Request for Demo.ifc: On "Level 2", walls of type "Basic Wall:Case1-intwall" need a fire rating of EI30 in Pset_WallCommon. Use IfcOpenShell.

First a look at what the model holds.

```python
import ifcopenshell
import ifcopenshell.util.element

model = ifcopenshell.open("Demo.ifc")
print(model.schema)
storey = next(s for s in model.by_type("IfcBuildingStorey") if s.Name == "Level 2")
walls = [e for e in ifcopenshell.util.element.get_decomposition(storey) if e.is_a("IfcWall")]
seen = {}
for e in walls:
    element_type = ifcopenshell.util.element.get_type(e)
    key = (element_type.Name if element_type != e and element_type else None, ifcopenshell.util.element.get_pset(e, "Pset_WallCommon", "FireRating"))
    seen[key] = seen.get(key, 0) + 1
for (name, value), count in sorted(seen.items(), key=str):
    print(count, "x", name, "|", value)
```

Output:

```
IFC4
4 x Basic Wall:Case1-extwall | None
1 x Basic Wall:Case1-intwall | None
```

```python
import ifcopenshell
import ifcopenshell.api.pset
import ifcopenshell.util.element

model = ifcopenshell.open("Demo.ifc")

storey = next(s for s in model.by_type("IfcBuildingStorey") if s.Name == "Level 2")
walls = [e for e in ifcopenshell.util.element.get_decomposition(storey) if e.is_a("IfcWall")]

count = 0
for e in walls:
    element_type = ifcopenshell.util.element.get_type(e)
    if element_type in (None, e) or element_type.Name != "Basic Wall:Case1-intwall":
        continue
    # add_pset returns the element's existing set when there is one.
    pset = ifcopenshell.api.pset.add_pset(model, product=e, name="Pset_WallCommon")
    ifcopenshell.api.pset.edit_pset(model, pset=pset, properties={"FireRating": "EI30"})
    count += 1

print(count, "walls updated")

model.write("Demo_updated.ifc")
```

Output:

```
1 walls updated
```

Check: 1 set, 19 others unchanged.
